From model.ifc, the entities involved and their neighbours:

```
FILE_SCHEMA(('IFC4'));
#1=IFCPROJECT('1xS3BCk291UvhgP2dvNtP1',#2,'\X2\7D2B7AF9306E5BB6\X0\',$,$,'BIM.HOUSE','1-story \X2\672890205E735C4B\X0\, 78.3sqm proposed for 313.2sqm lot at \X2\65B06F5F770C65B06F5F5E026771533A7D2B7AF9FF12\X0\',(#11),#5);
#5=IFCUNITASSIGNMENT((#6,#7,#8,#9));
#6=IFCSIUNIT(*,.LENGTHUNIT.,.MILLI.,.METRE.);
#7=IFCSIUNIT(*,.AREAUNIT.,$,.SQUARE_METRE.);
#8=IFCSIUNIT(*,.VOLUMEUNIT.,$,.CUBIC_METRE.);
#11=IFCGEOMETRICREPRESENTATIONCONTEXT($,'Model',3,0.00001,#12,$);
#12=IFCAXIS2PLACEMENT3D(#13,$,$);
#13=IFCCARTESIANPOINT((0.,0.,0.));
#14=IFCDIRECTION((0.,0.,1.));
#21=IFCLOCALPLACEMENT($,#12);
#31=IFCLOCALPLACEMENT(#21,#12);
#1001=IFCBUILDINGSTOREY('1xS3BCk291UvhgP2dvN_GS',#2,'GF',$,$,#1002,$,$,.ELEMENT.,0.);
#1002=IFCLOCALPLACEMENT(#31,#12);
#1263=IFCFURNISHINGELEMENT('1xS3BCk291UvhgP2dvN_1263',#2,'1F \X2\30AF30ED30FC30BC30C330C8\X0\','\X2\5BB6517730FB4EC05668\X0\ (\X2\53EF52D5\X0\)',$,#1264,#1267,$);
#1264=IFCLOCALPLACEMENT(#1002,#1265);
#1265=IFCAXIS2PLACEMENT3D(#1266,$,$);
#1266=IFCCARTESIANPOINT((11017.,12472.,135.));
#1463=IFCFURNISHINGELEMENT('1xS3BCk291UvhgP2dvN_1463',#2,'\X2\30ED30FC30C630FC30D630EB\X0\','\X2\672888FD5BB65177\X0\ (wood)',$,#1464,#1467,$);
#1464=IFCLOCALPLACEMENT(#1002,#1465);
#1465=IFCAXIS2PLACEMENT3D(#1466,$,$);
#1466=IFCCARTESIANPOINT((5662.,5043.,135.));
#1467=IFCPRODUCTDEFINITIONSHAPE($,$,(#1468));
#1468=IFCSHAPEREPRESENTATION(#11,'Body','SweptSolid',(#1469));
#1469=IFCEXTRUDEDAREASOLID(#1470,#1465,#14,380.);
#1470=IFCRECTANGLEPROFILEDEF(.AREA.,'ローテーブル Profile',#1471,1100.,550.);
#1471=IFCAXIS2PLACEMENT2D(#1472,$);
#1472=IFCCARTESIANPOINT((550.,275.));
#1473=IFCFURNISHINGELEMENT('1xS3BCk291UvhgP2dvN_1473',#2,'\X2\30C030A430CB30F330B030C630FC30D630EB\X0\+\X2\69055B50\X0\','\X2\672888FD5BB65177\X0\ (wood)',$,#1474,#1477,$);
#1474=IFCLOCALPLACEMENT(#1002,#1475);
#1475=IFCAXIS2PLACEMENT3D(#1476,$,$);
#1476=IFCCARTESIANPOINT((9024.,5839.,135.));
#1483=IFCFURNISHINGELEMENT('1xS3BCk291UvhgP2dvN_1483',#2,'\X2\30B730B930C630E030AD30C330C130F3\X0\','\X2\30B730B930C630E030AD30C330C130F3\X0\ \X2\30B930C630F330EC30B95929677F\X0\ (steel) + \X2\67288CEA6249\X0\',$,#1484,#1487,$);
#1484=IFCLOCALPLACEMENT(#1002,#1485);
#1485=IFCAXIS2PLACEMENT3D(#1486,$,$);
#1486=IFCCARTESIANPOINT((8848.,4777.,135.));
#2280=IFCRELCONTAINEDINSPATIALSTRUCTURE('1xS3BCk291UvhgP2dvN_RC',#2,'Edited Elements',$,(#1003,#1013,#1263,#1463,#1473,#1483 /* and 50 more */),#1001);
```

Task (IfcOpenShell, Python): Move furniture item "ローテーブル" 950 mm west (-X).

```python
import ifcopenshell
import ifcopenshell.api.geometry
import ifcopenshell.util.placement
import ifcopenshell.util.unit

model = ifcopenshell.open("model.ifc")
unit_scale = ifcopenshell.util.unit.calculate_unit_scale(model)

item = model.by_id(1463)
matrix = ifcopenshell.util.placement.get_local_placement(item.ObjectPlacement)
matrix[0, 3] -= 0.95 / unit_scale
ifcopenshell.api.geometry.edit_object_placement(model, product=item, matrix=matrix, is_si=False)

print(ifcopenshell.util.placement.get_local_placement(item.ObjectPlacement).round(3) + 0.0)

model.write("model_rev.ifc")
```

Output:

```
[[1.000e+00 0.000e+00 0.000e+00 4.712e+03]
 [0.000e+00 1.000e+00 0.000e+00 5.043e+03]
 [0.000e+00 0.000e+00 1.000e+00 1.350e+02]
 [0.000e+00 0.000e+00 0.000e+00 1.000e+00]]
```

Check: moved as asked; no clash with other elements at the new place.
